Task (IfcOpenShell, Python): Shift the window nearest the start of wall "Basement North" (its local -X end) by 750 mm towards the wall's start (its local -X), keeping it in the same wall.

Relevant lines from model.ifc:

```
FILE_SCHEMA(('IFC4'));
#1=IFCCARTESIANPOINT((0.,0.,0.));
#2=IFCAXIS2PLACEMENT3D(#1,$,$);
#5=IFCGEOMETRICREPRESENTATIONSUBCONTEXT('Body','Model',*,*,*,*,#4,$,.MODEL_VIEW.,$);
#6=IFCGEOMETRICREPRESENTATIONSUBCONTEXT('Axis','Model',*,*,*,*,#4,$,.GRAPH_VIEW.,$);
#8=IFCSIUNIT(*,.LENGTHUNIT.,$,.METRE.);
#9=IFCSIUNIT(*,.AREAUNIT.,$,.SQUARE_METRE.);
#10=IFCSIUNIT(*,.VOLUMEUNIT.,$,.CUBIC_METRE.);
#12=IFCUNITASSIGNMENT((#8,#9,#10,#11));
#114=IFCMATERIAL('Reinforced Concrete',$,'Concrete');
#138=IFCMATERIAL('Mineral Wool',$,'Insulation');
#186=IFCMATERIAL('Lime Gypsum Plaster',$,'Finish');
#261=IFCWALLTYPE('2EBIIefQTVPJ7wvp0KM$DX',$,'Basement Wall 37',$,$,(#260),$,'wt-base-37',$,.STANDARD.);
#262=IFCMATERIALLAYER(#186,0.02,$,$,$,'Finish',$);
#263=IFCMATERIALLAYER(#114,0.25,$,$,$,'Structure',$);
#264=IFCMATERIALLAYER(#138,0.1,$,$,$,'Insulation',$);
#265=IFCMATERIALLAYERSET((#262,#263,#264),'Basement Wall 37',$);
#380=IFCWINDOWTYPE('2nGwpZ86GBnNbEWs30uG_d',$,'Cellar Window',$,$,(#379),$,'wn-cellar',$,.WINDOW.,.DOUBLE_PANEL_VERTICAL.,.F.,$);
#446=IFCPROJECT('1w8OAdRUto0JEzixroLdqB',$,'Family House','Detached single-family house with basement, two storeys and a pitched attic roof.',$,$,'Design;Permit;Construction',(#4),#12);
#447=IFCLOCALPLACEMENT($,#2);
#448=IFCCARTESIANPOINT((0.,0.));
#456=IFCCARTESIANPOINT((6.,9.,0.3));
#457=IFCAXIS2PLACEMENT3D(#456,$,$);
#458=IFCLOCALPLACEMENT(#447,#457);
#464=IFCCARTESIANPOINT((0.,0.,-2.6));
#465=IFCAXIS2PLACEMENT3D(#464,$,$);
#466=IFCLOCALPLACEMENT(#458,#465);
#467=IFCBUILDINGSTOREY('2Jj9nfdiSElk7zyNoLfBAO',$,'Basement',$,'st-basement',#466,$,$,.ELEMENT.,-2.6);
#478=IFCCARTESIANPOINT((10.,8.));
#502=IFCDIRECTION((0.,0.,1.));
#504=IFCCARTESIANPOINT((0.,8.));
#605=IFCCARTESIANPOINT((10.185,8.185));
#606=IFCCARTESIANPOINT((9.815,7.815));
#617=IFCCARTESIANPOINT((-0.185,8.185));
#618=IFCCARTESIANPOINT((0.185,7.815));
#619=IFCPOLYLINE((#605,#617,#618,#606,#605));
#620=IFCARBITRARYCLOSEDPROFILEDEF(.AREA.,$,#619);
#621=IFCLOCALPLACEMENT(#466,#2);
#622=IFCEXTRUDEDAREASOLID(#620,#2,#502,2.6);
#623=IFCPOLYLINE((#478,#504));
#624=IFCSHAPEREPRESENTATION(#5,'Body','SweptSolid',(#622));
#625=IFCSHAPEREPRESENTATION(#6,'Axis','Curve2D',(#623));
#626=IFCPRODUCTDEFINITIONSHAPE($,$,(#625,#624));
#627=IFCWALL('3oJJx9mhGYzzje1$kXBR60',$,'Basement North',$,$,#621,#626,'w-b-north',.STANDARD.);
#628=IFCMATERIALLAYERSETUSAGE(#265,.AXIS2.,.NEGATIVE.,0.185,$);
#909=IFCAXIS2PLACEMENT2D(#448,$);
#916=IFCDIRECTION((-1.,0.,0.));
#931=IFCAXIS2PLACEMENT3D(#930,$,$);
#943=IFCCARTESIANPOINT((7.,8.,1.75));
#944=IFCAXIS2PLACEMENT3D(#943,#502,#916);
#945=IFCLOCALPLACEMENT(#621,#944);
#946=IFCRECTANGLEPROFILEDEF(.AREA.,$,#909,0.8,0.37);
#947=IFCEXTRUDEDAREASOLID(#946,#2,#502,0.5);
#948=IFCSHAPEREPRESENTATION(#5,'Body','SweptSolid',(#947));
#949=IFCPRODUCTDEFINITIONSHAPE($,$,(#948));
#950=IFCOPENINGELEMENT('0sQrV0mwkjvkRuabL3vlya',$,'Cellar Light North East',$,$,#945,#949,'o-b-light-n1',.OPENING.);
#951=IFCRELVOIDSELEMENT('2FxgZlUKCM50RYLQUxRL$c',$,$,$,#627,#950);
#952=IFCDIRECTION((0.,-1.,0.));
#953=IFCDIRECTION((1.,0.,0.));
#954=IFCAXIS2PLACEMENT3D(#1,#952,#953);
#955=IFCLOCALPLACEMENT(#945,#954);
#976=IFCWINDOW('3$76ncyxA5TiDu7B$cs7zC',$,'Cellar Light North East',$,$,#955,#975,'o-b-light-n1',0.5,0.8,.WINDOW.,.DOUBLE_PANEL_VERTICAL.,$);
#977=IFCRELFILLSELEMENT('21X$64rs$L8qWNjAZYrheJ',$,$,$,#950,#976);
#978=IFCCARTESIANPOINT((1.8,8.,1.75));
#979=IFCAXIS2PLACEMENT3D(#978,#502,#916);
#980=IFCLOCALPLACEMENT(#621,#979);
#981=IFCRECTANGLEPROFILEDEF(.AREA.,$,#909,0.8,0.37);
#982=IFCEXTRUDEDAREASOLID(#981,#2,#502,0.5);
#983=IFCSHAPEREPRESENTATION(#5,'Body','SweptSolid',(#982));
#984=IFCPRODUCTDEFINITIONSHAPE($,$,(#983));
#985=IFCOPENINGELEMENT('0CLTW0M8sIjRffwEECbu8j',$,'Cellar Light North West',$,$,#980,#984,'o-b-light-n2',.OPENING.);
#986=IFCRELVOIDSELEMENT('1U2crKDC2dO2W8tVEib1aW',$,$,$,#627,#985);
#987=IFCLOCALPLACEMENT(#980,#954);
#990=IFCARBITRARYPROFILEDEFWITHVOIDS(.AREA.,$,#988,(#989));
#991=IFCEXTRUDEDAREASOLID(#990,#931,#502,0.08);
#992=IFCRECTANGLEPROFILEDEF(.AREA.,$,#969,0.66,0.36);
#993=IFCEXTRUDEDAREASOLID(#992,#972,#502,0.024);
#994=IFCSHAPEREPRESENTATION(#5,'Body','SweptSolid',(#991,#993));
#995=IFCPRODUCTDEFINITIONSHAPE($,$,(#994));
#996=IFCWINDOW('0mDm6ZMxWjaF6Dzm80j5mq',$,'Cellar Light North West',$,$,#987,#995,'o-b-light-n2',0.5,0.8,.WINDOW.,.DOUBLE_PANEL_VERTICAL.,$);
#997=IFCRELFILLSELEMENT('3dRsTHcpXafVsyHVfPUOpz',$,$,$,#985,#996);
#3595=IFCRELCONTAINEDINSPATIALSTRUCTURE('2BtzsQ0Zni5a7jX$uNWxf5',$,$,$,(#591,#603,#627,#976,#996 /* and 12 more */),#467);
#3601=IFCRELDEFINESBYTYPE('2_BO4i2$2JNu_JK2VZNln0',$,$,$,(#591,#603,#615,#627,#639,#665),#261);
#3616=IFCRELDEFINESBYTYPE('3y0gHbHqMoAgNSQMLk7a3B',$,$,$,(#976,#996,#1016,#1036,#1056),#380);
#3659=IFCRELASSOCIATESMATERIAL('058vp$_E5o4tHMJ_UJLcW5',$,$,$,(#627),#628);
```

```python
import ifcopenshell
import ifcopenshell.api.geometry
import ifcopenshell.util.placement
import ifcopenshell.util.unit

model = ifcopenshell.open("model.ifc")
unit_scale = ifcopenshell.util.unit.calculate_unit_scale(model)

window = model.by_id(996)
opening = window.FillsVoids[0].RelatingOpeningElement
wall = opening.VoidsElements[0].RelatingBuildingElement

wall_matrix = ifcopenshell.util.placement.get_local_placement(wall.ObjectPlacement)
shift = wall_matrix[:3, 0] * -0.75 / unit_scale
before = ifcopenshell.util.placement.get_local_placement(window.ObjectPlacement)[:3, 3].copy()

# The window is placed relative to its opening, so it follows when the opening moves.
matrix = ifcopenshell.util.placement.get_local_placement(opening.ObjectPlacement)
matrix[:3, 3] += shift
ifcopenshell.api.geometry.edit_object_placement(
    model, product=opening, matrix=matrix, is_si=False, should_transform_children=True
)

after = ifcopenshell.util.placement.get_local_placement(window.ObjectPlacement)[:3, 3]
print("window moved by", (after - before).round(3) + 0.0)

model.write("model_updated.ifc")
```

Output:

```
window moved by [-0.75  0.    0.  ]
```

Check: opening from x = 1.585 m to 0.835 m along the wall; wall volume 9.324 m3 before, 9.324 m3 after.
